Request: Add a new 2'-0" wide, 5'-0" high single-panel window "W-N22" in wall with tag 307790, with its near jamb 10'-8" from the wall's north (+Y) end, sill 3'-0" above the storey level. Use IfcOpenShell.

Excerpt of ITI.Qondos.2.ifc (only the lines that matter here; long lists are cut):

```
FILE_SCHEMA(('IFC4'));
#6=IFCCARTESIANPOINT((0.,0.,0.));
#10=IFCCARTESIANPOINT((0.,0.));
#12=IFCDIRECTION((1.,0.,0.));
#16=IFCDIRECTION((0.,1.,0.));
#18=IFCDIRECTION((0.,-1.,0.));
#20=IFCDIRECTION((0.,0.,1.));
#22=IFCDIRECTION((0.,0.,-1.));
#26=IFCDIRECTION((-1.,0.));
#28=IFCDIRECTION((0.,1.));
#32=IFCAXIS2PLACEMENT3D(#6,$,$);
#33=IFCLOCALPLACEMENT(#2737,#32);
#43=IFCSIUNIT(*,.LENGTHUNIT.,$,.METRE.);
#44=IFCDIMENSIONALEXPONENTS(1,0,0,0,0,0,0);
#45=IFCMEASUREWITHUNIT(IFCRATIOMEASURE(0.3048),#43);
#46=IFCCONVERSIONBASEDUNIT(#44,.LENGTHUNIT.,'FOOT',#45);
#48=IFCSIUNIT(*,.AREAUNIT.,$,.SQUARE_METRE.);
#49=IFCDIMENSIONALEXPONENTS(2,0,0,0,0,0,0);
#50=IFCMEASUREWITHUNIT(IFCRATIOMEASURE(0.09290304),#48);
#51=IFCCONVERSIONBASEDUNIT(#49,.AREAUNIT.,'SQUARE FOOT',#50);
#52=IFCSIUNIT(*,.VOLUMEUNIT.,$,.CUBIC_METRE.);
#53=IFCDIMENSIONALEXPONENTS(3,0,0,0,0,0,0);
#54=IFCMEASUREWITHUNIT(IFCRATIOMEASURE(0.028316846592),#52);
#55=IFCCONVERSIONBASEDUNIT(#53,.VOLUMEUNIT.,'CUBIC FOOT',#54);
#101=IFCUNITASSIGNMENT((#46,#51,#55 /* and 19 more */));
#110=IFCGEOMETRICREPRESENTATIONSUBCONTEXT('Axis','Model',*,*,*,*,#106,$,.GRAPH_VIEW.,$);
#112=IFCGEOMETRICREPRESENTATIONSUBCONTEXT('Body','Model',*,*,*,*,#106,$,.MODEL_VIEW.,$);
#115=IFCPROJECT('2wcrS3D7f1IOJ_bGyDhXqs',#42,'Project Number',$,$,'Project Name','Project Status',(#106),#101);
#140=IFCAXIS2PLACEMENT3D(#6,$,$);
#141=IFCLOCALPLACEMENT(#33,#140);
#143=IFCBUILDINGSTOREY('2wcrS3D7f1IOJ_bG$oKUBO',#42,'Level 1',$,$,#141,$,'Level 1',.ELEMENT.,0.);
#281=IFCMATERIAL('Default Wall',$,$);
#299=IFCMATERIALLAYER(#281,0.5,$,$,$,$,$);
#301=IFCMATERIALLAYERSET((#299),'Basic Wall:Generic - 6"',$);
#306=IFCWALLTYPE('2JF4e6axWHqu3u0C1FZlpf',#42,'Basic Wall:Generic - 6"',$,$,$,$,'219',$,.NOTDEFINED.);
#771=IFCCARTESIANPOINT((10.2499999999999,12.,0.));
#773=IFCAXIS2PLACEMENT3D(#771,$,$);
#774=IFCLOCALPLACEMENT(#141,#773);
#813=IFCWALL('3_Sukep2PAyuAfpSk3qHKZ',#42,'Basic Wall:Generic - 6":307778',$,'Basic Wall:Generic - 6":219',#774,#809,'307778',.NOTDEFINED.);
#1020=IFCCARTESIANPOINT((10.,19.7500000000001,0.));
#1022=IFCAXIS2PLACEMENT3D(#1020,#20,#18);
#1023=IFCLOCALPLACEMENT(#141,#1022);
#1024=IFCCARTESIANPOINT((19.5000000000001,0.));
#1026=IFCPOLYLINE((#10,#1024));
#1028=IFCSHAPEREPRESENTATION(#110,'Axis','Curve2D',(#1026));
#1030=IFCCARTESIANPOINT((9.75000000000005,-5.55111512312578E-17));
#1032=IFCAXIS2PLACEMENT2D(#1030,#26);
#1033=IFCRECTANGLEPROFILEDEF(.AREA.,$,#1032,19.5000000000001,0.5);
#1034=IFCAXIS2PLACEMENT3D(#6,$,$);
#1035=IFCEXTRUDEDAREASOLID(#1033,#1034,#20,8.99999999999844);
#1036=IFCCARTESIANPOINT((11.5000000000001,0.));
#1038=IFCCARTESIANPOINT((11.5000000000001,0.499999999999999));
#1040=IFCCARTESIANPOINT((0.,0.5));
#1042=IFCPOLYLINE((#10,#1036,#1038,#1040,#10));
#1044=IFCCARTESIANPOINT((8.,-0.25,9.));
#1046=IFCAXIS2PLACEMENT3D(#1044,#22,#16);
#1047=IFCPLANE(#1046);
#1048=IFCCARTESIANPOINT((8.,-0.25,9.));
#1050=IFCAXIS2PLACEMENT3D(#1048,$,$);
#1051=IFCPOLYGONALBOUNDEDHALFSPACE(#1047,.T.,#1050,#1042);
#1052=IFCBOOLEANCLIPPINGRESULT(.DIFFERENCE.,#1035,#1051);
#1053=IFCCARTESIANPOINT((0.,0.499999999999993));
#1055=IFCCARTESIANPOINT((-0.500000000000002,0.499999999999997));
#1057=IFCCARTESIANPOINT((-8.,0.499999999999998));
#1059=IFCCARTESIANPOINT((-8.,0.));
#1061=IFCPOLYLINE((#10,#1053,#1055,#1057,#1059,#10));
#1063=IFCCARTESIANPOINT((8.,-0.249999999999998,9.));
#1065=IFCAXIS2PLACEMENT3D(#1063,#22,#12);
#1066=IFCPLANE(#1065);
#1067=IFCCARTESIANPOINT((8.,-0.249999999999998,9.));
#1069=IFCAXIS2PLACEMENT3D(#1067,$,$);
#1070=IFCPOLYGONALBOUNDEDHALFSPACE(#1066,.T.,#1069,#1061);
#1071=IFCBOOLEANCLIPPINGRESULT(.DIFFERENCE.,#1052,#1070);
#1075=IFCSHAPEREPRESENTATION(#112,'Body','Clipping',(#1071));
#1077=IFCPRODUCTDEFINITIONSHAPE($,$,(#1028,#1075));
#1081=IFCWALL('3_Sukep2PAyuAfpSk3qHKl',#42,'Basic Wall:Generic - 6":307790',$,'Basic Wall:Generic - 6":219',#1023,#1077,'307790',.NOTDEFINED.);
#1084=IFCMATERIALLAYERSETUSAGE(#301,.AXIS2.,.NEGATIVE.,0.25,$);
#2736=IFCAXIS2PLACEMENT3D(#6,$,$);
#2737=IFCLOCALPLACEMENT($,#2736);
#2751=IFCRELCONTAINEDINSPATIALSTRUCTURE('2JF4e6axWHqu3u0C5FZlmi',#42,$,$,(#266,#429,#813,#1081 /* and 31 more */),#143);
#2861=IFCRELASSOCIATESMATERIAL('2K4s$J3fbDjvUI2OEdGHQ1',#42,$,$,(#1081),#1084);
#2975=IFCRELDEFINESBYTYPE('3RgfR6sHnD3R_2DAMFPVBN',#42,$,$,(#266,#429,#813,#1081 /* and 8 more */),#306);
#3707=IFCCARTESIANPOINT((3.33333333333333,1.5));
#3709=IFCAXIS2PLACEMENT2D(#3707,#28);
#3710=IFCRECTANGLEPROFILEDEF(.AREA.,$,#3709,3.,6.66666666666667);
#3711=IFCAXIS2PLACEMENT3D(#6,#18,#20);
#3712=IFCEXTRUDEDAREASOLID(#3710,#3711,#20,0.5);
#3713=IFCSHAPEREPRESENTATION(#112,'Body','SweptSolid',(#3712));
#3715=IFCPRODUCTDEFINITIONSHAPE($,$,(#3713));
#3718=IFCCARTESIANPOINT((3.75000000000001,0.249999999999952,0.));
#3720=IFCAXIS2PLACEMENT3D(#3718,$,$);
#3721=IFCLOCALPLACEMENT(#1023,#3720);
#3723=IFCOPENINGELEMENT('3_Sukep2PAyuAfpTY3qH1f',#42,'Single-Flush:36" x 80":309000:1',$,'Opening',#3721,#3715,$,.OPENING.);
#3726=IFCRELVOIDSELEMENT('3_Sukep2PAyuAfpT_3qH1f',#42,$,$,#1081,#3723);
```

```python
import numpy as np
import ifcopenshell
import ifcopenshell.api.feature
import ifcopenshell.api.geometry
import ifcopenshell.api.root
import ifcopenshell.api.spatial
import ifcopenshell.geom
import ifcopenshell.util.element
import ifcopenshell.util.placement
import ifcopenshell.util.representation
import ifcopenshell.util.shape
import ifcopenshell.util.unit

model = ifcopenshell.open("ITI.Qondos.2.ifc")
unit_scale = ifcopenshell.util.unit.calculate_unit_scale(model)
settings = ifcopenshell.geom.settings()


def volume(element):
    """Net volume in cubic metres, openings subtracted."""
    shape = ifcopenshell.geom.create_shape(settings, element)
    return ifcopenshell.util.shape.get_volume(shape.geometry)


wall = model.by_id(1081)
storey = ifcopenshell.util.element.get_container(wall, ifc_class="IfcBuildingStorey")
context = ifcopenshell.util.representation.get_context(model, "Model", "Body", "MODEL_VIEW")
before = volume(wall)

width, height, from_end, sill = 0.6096, 1.524, 3.2512, 0.9144  # metres

# The wall runs along its own X axis, and the end named is its -X end.
wall_shape = ifcopenshell.geom.create_shape(settings, wall)
x, y, z = ifcopenshell.util.shape.get_vertices(wall_shape.geometry).T
start = x.min() + from_end
face, thickness = float(y.min()), float(y.max() - y.min())
wall_matrix = ifcopenshell.util.placement.get_local_placement(wall.ObjectPlacement)
level = ifcopenshell.util.placement.get_local_placement(storey.ObjectPlacement)[2, 3]


def in_wall(x, y):
    """Placement at x, y metres in the wall's axes, at sill height."""
    matrix = wall_matrix.copy()
    matrix[:, 3] = wall_matrix @ np.array([x / unit_scale, y / unit_scale, 0.0, 1.0])
    matrix[2, 3] = level + sill / unit_scale
    return matrix


# Opening: a box that overshoots both wall faces by 50 mm.
opening = ifcopenshell.api.root.create_entity(model, ifc_class="IfcOpeningElement", predefined_type="OPENING")
box = ifcopenshell.api.geometry.add_wall_representation(
    model, context=context, length=width, height=height, thickness=thickness + 0.1
)
ifcopenshell.api.geometry.assign_representation(model, product=opening, representation=box)
ifcopenshell.api.geometry.edit_object_placement(model, product=opening, matrix=in_wall(start, face - 0.05), is_si=False)
ifcopenshell.api.feature.add_feature(model, feature=opening, element=wall)

window = ifcopenshell.api.root.create_entity(model, ifc_class="IfcWindow", name="W-N22", predefined_type="WINDOW")
window.OverallWidth, window.OverallHeight = width / unit_scale, height / unit_scale
window.PartitioningType = "SINGLE_PANEL"
body = ifcopenshell.api.geometry.add_window_representation(
    model,
    context=context,
    overall_width=window.OverallWidth,
    overall_height=window.OverallHeight,
    partition_type="SINGLE_PANEL",
)
ifcopenshell.api.geometry.assign_representation(model, product=window, representation=body)
ifcopenshell.api.spatial.assign_container(model, products=[window], relating_structure=storey)
ifcopenshell.api.feature.add_filling(model, opening=opening, element=window)

# Centre the window in the wall's thickness.
ifcopenshell.api.geometry.edit_object_placement(model, product=window, matrix=in_wall(start, face), is_si=False)
window_shape = ifcopenshell.geom.create_shape(settings, window)
depth = ifcopenshell.util.shape.get_vertices(window_shape.geometry)[:, 1]
offset = face + thickness / 2 - (depth.min() + depth.max()) / 2
ifcopenshell.api.geometry.edit_object_placement(model, product=window, matrix=in_wall(start, offset), is_si=False)

after = volume(wall)

print(f"wall volume {before:.3f} -> {after:.3f} m3")

model.write("ITI.Qondos.2_edited.ifc")
```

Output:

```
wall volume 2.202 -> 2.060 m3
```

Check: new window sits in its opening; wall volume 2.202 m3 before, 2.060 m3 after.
